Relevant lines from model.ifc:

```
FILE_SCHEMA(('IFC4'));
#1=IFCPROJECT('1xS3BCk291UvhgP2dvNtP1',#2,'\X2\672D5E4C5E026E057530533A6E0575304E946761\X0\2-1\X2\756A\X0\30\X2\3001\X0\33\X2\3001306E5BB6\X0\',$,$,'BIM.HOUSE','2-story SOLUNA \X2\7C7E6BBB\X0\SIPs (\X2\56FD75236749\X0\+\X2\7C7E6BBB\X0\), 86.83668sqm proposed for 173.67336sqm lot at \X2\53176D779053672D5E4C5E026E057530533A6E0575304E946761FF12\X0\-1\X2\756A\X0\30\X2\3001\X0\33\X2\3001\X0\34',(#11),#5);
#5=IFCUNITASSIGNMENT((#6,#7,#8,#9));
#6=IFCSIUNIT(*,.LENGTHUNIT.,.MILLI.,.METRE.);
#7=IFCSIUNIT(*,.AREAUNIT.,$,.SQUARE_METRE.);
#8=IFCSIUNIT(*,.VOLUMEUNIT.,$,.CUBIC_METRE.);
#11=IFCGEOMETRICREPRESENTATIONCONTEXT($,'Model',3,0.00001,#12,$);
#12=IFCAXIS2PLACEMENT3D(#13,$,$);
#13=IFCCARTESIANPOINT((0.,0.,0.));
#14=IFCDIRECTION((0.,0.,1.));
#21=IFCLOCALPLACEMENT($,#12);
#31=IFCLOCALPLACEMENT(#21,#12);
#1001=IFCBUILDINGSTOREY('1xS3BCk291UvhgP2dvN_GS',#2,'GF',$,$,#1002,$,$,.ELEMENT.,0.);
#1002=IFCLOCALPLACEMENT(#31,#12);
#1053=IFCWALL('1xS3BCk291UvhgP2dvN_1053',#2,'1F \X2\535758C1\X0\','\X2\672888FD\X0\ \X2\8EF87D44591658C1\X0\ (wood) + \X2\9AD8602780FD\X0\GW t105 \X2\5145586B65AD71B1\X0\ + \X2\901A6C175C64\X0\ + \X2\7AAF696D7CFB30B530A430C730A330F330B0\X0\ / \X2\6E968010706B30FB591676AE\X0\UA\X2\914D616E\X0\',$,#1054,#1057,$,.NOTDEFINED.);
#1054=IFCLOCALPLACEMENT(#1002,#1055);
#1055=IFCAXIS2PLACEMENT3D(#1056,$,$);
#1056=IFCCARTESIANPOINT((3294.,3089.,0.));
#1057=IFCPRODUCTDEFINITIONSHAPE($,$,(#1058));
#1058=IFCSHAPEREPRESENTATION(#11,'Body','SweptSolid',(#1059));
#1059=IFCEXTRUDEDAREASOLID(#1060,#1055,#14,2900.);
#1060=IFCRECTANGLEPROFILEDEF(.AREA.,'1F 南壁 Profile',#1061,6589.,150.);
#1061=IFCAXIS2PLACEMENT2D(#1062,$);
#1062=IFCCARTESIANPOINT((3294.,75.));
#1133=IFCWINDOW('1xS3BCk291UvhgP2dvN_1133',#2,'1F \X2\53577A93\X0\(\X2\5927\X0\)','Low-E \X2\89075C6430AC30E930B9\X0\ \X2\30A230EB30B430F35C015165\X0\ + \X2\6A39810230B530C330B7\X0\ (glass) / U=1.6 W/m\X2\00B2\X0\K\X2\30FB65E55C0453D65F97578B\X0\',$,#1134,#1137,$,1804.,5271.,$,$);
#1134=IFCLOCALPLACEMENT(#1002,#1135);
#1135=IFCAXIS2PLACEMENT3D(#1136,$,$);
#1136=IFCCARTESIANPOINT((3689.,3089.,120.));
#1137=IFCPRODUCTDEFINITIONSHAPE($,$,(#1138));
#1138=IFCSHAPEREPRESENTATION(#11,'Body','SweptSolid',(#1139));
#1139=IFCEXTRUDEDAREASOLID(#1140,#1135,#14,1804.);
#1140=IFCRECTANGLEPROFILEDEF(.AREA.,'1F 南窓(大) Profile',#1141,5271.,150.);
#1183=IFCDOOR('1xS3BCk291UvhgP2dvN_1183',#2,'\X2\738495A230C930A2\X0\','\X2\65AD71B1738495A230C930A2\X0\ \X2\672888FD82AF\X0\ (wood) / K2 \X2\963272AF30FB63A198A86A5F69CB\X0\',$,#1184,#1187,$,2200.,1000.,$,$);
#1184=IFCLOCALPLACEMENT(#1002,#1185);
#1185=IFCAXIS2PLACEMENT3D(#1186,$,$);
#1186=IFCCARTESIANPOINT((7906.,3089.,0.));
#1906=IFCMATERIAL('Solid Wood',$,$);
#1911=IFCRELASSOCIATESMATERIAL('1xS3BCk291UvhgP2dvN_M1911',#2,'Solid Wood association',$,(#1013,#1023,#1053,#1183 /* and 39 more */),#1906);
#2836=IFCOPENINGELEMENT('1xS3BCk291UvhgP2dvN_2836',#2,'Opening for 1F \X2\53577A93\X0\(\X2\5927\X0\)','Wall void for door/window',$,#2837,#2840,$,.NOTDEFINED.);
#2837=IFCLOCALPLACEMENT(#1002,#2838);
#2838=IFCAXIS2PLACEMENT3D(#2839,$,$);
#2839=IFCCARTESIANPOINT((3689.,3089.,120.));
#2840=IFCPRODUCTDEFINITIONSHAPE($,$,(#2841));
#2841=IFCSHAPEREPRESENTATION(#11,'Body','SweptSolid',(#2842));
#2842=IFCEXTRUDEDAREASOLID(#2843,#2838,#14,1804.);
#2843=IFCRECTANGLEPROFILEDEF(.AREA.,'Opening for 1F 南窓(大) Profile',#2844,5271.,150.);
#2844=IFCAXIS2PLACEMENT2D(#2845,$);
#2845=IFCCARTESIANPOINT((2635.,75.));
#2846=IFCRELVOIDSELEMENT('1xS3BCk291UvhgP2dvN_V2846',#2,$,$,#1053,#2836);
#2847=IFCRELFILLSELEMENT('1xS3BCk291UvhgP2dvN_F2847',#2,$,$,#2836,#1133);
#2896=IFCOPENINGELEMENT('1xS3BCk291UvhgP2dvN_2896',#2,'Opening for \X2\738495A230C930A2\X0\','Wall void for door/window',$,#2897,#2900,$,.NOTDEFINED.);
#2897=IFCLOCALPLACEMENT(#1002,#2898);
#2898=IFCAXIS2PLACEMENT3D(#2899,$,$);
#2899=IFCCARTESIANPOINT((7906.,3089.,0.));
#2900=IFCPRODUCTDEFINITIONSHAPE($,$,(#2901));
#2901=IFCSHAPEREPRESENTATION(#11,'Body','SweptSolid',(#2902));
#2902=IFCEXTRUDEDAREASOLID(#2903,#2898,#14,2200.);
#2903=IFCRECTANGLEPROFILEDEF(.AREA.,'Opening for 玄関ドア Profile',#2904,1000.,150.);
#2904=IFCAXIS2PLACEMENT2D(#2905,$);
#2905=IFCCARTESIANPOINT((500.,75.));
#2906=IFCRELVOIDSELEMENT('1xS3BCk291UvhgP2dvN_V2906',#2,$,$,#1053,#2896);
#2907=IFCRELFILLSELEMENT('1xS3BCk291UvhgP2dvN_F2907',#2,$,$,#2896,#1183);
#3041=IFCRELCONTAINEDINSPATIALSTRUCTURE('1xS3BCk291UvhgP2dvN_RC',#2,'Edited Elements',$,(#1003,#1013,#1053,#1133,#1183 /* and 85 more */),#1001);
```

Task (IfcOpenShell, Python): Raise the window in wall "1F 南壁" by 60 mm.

```python
import numpy as np
import ifcopenshell
import ifcopenshell.api.geometry
import ifcopenshell.util.placement
import ifcopenshell.util.unit

model = ifcopenshell.open("model.ifc")
unit_scale = ifcopenshell.util.unit.calculate_unit_scale(model)

window = model.by_guid("1xS3BCk291UvhgP2dvN_1133")
opening = window.FillsVoids[0].RelatingOpeningElement
dz = 60.0

shift = np.array([0.0, 0.0, dz])
# The window is not placed relative to its opening, so move both.
for product in (opening, window):
    matrix = ifcopenshell.util.placement.get_local_placement(product.ObjectPlacement)
    matrix[:3, 3] += shift
    ifcopenshell.api.geometry.edit_object_placement(model, product=product, matrix=matrix, is_si=False)

print(f"moved by {dz * unit_scale:+.3f} m")

model.write("model-out.ifc")
```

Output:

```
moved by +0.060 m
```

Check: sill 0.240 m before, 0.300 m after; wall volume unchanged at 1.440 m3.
